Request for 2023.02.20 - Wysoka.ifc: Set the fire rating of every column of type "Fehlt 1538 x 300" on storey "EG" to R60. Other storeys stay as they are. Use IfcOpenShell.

First a look at what the model holds.

```python
import ifcopenshell
import ifcopenshell.util.element

model = ifcopenshell.open("2023.02.20 - Wysoka.ifc")
print(model.schema)
storey = next(s for s in model.by_type("IfcBuildingStorey") if s.Name == "EG")
columns = [e for e in ifcopenshell.util.element.get_decomposition(storey) if e.is_a("IfcColumn")]
seen = {}
for e in columns:
    element_type = ifcopenshell.util.element.get_type(e)
    key = (element_type.Name if element_type != e and element_type else None, ifcopenshell.util.element.get_pset(e, "Pset_ColumnCommon", "FireRating"))
    seen[key] = seen.get(key, 0) + 1
for (name, value), count in sorted(seen.items(), key=str):
    print(count, "x", name, "|", value)
```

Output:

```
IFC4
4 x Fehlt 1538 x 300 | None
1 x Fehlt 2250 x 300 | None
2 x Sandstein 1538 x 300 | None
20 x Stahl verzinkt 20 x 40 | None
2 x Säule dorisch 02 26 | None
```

```python
import ifcopenshell
import ifcopenshell.api.pset
import ifcopenshell.util.element

model = ifcopenshell.open("2023.02.20 - Wysoka.ifc")

storey = next(s for s in model.by_type("IfcBuildingStorey") if s.Name == "EG")
columns = [e for e in ifcopenshell.util.element.get_decomposition(storey) if e.is_a("IfcColumn")]

count = 0
for e in columns:
    element_type = ifcopenshell.util.element.get_type(e)
    if element_type in (None, e) or element_type.Name != "Fehlt 1538 x 300":
        continue
    # add_pset returns the element's existing set when there is one.
    pset = ifcopenshell.api.pset.add_pset(model, product=e, name="Pset_ColumnCommon")
    ifcopenshell.api.pset.edit_pset(model, pset=pset, properties={"FireRating": "R60"})
    count += 1

print(count, "columns updated")

model.write("2023.02.20 - Wysoka_v2.ifc")
```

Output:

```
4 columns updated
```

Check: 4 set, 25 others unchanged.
